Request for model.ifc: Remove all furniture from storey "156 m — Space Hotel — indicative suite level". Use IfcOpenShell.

First a look at what the model holds.

```python
import ifcopenshell
import ifcopenshell.util.element

model = ifcopenshell.open("model.ifc")
print(model.schema)
storey = next(s for s in model.by_type("IfcBuildingStorey") if s.Name == "156 m — Space Hotel — indicative suite level")
furniture = [e for e in ifcopenshell.util.element.get_decomposition(storey) if e.is_a("IfcFurnishingElement")]
seen = {}
for e in furniture:
    element_type = ifcopenshell.util.element.get_type(e)
    name = element_type.Name if element_type not in (None, e) else None
    seen[name] = seen.get(name, 0) + 1
for name, count in sorted(seen.items(), key=str):
    print(count, "x", name)
```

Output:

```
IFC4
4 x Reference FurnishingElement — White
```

```python
import ifcopenshell
import ifcopenshell.api.root
import ifcopenshell.util.element

model = ifcopenshell.open("model.ifc")

storey = next(s for s in model.by_type("IfcBuildingStorey") if s.Name == "156 m — Space Hotel — indicative suite level")
furniture = [e for e in ifcopenshell.util.element.get_decomposition(storey) if e.is_a("IfcFurnishingElement")]

for e in furniture:
    ifcopenshell.api.root.remove_product(model, product=e)
print(len(furniture), "removed")

model.write("model-out.ifc")
```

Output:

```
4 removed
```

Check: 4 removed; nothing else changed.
